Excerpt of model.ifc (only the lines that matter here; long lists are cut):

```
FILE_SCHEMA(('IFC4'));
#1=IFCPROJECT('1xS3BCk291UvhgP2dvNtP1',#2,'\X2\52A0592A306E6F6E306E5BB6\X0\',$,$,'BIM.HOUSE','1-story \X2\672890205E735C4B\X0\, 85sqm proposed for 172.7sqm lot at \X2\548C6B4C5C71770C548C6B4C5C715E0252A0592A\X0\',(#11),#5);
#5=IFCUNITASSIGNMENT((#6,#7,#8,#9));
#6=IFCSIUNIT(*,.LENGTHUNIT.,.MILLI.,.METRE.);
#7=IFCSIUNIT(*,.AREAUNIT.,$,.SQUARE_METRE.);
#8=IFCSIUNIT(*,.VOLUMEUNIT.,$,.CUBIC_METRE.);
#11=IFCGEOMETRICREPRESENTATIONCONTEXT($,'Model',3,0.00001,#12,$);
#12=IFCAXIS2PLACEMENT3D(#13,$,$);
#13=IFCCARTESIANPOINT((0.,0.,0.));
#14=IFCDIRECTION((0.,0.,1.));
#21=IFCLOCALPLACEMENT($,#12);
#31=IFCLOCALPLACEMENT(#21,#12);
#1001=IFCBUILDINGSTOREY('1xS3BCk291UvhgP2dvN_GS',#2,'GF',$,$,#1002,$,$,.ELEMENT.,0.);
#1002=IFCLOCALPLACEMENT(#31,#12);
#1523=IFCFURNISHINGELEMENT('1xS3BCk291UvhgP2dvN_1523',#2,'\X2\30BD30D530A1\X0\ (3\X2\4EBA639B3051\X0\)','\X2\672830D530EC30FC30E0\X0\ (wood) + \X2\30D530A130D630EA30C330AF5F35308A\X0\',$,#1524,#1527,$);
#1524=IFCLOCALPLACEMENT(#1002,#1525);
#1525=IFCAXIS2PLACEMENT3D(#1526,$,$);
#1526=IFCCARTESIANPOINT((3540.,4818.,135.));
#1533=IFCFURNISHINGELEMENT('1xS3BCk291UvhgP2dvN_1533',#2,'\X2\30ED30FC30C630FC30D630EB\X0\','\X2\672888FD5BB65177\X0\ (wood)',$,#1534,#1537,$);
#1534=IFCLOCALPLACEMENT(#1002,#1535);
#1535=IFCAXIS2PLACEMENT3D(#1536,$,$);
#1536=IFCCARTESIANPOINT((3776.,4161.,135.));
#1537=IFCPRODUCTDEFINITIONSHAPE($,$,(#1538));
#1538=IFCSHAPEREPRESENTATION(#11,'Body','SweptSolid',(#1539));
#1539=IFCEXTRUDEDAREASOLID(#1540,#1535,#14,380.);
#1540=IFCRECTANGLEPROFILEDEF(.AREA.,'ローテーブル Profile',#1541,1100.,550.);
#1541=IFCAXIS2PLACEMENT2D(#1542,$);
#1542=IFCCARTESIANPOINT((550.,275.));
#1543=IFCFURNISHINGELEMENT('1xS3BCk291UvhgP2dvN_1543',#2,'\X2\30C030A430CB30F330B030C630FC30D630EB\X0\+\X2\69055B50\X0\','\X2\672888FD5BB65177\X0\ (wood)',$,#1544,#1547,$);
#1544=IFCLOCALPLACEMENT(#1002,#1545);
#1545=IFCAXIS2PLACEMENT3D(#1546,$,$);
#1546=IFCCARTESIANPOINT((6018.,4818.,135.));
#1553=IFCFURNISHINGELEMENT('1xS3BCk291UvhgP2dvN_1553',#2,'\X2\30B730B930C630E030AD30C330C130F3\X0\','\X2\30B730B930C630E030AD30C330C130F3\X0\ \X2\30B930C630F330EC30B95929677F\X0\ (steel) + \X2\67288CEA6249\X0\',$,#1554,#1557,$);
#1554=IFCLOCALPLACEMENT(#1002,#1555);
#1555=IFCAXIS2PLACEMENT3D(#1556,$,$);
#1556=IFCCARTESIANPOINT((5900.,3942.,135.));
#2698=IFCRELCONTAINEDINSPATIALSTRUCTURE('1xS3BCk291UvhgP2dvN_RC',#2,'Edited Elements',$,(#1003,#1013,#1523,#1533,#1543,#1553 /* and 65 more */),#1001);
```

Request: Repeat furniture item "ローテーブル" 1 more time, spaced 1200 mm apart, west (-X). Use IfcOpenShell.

```python
import numpy as np
import ifcopenshell
import ifcopenshell.api.geometry
import ifcopenshell.api.root
import ifcopenshell.util.element
import ifcopenshell.util.placement
import ifcopenshell.util.unit

model = ifcopenshell.open("model.ifc")
unit_scale = ifcopenshell.util.unit.calculate_unit_scale(model)


def reuse_history(source, copy):
    """copy_class also copies each property set's owner history, people and application; keep the originals."""
    for rel in copy.IsDefinedBy:
        if rel.is_a("IfcRelDefinesByProperties") and (history := rel.RelatingPropertyDefinition.OwnerHistory):
            rel.RelatingPropertyDefinition.OwnerHistory = source.OwnerHistory
            ifcopenshell.util.element.remove_deep2(model, history)


source = model.by_guid("1xS3BCk291UvhgP2dvN_1533")
base = ifcopenshell.util.placement.get_local_placement(source.ObjectPlacement)
step = np.array([-1.0, 0.0, 0.0]) * 1.2 / unit_scale

for i in range(1, 2):
    copy = ifcopenshell.api.root.copy_class(model, product=source)
    copy.Representation = ifcopenshell.util.element.copy_deep(
        model, source.Representation, exclude=["IfcGeometricRepresentationContext", "IfcRepresentationMap"]
    )
    reuse_history(source, copy)
    matrix = base.copy()
    matrix[:3, 3] += i * step
    print("added at", matrix[:3, 3].round(3) + 0.0)
    ifcopenshell.api.geometry.edit_object_placement(model, product=copy, matrix=matrix, is_si=False)

model.write("model_rev.ifc")
```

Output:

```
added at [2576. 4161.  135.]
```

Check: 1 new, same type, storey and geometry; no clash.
